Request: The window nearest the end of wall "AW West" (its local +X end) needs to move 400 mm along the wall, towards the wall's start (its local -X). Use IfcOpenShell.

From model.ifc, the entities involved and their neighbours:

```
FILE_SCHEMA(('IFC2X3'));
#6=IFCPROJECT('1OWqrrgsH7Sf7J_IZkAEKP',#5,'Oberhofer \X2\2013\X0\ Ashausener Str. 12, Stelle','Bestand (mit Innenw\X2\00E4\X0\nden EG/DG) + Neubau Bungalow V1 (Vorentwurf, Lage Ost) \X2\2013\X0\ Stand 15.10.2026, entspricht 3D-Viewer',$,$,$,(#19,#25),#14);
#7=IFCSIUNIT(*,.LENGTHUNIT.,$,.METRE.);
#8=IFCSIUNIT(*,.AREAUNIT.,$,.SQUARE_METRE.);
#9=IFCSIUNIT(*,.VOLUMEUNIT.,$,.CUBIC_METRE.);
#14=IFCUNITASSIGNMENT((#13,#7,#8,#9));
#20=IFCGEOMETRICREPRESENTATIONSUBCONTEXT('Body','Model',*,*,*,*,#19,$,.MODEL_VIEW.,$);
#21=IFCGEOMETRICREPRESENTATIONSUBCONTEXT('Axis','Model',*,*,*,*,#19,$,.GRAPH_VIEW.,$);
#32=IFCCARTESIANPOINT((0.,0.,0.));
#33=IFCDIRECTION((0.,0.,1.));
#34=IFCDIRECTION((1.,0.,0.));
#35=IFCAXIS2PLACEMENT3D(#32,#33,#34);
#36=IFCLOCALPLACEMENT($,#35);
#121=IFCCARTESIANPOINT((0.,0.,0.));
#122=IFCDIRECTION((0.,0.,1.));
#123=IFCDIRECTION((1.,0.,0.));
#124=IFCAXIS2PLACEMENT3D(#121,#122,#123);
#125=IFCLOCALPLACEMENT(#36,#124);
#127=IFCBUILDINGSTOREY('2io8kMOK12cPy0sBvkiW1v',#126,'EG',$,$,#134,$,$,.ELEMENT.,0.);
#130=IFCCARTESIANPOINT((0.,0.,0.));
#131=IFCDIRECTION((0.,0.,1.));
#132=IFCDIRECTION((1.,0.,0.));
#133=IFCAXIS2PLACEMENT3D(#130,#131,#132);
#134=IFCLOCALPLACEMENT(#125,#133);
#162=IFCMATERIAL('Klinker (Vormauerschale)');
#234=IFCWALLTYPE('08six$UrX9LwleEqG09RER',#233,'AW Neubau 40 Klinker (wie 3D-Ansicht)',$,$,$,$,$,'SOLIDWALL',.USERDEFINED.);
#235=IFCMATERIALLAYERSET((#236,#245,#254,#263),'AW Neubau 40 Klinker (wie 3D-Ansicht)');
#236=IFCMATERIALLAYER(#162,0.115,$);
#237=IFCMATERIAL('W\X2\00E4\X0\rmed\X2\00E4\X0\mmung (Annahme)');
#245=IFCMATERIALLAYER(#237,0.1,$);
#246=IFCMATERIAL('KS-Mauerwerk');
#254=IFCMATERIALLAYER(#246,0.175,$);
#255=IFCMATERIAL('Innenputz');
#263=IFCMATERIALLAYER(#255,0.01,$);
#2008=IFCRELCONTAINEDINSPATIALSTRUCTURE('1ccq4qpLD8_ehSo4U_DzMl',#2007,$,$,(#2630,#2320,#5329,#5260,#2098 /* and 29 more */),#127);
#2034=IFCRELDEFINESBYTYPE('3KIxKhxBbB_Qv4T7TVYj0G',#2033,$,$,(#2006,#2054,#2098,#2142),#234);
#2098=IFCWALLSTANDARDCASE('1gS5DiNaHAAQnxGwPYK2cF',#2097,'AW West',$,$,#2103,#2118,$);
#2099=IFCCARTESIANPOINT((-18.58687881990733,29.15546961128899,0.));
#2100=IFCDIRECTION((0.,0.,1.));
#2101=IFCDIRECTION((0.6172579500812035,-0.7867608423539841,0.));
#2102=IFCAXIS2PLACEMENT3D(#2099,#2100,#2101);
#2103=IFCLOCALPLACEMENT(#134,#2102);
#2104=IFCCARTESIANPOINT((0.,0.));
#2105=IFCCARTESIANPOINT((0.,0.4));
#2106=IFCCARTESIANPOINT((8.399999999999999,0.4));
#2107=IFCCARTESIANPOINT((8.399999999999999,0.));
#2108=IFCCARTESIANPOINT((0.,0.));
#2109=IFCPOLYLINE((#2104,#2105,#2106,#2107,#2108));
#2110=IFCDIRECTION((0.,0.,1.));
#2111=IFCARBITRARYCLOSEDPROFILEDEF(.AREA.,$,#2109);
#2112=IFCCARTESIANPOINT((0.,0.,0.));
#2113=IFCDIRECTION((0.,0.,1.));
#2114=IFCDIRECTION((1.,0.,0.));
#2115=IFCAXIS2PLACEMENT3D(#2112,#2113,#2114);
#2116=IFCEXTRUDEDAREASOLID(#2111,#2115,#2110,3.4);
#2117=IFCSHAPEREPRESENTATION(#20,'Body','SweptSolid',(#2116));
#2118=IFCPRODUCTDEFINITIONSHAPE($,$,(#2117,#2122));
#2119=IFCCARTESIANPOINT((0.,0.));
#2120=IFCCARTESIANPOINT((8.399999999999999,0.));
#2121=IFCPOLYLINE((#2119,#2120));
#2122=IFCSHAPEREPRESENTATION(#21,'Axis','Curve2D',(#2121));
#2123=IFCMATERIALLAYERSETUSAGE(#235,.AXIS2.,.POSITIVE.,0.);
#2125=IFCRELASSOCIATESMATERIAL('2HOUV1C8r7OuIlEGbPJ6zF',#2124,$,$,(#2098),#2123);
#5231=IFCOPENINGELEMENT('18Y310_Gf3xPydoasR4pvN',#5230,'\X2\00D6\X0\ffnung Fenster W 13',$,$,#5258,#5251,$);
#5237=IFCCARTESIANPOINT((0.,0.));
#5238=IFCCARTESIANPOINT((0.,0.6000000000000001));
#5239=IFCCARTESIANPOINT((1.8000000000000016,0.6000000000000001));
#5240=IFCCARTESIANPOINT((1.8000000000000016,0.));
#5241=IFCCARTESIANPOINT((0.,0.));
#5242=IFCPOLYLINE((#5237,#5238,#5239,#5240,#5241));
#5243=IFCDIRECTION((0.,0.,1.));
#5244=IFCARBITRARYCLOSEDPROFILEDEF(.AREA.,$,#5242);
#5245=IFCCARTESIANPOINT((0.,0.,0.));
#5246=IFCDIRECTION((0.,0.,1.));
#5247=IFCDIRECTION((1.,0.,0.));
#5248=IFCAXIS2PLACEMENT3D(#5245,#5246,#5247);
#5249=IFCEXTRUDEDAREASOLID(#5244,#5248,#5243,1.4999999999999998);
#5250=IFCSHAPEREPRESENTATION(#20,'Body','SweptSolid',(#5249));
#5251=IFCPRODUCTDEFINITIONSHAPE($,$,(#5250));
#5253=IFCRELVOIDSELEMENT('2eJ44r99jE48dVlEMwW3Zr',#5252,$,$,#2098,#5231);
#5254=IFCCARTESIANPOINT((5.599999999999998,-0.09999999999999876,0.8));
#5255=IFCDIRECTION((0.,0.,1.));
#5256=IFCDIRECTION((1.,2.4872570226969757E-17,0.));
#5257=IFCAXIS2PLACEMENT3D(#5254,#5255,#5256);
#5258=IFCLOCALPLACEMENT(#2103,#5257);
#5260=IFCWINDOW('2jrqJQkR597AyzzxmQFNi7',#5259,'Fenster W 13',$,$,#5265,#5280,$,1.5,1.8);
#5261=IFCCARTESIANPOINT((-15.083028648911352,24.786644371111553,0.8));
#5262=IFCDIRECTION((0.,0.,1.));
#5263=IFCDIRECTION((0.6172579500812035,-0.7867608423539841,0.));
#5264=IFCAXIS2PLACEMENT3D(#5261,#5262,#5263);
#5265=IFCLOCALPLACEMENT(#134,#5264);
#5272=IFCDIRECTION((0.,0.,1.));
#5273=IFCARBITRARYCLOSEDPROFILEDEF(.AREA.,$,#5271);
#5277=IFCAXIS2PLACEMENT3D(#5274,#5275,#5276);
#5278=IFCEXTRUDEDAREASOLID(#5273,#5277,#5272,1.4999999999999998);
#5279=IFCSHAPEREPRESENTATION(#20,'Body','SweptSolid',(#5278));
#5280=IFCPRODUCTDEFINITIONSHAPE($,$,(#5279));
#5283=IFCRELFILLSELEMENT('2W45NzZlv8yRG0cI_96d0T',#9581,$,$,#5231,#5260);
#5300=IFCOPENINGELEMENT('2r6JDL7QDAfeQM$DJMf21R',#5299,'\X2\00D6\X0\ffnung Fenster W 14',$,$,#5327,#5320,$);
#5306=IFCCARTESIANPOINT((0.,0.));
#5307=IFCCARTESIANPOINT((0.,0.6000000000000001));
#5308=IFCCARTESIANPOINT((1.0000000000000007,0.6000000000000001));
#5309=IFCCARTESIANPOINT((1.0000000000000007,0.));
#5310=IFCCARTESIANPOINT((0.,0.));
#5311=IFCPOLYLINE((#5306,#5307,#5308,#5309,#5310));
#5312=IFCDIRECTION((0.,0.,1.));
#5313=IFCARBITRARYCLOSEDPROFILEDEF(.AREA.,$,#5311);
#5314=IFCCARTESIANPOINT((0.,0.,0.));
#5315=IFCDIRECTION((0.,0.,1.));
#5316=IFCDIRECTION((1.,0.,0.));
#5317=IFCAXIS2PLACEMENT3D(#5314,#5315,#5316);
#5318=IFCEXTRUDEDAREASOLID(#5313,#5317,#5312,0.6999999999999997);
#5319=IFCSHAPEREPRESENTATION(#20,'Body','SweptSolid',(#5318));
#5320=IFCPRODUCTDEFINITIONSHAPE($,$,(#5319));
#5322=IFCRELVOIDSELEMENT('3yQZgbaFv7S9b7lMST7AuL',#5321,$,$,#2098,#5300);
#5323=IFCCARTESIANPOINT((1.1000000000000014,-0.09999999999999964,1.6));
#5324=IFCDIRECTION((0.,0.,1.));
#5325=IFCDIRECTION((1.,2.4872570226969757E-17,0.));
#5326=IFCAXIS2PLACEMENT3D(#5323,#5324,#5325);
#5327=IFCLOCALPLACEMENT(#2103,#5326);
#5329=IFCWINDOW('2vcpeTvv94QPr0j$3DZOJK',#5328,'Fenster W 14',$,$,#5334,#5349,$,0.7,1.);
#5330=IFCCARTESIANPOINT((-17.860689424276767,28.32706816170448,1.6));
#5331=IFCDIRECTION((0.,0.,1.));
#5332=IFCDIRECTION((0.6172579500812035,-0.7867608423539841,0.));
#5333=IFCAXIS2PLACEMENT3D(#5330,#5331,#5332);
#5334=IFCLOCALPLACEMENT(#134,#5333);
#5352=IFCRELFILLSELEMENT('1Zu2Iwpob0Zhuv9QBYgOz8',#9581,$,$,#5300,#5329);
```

```python
import ifcopenshell
import ifcopenshell.api.geometry
import ifcopenshell.util.placement

model = ifcopenshell.open("model.ifc")

window = model.by_guid("2jrqJQkR597AyzzxmQFNi7")
opening = window.FillsVoids[0].RelatingOpeningElement
wall = opening.VoidsElements[0].RelatingBuildingElement

wall_matrix = ifcopenshell.util.placement.get_local_placement(wall.ObjectPlacement)
shift = wall_matrix[:3, 0] * -0.4
before = ifcopenshell.util.placement.get_local_placement(window.ObjectPlacement)[:3, 3].copy()

# The window is not placed relative to its opening, so move both.
for product in (opening, window):
    matrix = ifcopenshell.util.placement.get_local_placement(product.ObjectPlacement)
    matrix[:3, 3] += shift
    ifcopenshell.api.geometry.edit_object_placement(model, product=product, matrix=matrix, is_si=False)

after = ifcopenshell.util.placement.get_local_placement(window.ObjectPlacement)[:3, 3]
print("window moved by", (after - before).round(3) + 0.0)

model.write("model_edited.ifc")
```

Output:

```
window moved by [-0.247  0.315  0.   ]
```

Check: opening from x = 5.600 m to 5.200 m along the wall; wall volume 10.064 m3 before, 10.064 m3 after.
